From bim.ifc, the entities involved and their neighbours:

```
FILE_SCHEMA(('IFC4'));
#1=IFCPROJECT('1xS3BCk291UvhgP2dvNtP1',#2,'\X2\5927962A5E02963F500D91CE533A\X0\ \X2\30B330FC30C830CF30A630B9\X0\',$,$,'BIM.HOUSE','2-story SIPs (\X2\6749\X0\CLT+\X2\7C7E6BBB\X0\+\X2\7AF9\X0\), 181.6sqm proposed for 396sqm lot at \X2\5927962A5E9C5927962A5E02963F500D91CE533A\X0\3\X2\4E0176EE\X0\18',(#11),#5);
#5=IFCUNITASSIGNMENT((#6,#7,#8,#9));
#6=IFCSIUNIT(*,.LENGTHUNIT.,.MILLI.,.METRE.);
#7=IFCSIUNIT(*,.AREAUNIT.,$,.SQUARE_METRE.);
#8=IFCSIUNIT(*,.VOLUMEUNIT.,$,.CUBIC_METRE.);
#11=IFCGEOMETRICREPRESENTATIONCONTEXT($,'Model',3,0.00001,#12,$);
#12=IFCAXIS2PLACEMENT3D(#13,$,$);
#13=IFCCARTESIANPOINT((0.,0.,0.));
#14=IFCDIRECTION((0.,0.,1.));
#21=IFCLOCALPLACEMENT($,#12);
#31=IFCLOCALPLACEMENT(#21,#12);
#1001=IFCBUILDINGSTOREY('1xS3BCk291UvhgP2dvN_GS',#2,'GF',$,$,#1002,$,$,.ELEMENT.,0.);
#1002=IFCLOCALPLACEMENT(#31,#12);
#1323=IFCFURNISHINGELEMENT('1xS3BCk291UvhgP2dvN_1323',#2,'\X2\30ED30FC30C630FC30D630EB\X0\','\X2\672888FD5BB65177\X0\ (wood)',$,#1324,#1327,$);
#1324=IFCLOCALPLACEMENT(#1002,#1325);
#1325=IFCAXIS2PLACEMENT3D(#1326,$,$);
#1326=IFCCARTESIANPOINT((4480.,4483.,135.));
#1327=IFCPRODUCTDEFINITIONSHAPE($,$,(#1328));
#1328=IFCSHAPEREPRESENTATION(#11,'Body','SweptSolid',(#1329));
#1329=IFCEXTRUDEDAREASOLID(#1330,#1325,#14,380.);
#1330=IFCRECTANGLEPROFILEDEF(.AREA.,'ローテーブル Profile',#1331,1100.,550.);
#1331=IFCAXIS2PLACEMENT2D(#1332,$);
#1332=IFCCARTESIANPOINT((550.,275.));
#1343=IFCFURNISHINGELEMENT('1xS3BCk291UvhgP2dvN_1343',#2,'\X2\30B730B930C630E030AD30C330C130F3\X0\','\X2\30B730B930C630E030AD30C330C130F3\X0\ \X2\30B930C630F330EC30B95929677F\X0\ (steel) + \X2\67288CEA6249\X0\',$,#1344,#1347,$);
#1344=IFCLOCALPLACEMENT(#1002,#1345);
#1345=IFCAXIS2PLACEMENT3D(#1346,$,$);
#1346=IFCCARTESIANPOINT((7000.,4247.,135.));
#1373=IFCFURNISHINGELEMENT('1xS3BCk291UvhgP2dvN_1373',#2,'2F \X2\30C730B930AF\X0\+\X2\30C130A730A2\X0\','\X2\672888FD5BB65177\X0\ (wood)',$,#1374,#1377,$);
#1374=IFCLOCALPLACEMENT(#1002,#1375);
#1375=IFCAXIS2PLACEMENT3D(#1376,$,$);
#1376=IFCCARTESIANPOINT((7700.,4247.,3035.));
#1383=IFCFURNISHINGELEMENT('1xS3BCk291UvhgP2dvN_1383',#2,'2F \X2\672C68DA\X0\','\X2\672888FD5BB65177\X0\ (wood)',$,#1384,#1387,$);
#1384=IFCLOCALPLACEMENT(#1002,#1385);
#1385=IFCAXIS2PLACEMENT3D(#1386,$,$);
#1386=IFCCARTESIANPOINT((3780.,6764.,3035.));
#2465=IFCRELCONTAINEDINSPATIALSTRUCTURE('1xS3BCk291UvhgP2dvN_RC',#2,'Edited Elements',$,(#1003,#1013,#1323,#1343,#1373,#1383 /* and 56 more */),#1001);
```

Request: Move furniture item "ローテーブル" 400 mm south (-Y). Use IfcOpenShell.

```python
import ifcopenshell
import ifcopenshell.api.geometry
import ifcopenshell.util.placement

model = ifcopenshell.open("bim.ifc")

item = model.by_guid("1xS3BCk291UvhgP2dvN_1323")
matrix = ifcopenshell.util.placement.get_local_placement(item.ObjectPlacement)
matrix[1, 3] -= 400.0
ifcopenshell.api.geometry.edit_object_placement(model, product=item, matrix=matrix, is_si=False)

print(ifcopenshell.util.placement.get_local_placement(item.ObjectPlacement).round(3) + 0.0)

model.write("bim_edited.ifc")
```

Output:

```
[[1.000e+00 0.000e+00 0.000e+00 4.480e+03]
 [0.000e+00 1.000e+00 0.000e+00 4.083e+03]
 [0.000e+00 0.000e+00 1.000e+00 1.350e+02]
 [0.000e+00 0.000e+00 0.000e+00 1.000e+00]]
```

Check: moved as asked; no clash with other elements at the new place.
